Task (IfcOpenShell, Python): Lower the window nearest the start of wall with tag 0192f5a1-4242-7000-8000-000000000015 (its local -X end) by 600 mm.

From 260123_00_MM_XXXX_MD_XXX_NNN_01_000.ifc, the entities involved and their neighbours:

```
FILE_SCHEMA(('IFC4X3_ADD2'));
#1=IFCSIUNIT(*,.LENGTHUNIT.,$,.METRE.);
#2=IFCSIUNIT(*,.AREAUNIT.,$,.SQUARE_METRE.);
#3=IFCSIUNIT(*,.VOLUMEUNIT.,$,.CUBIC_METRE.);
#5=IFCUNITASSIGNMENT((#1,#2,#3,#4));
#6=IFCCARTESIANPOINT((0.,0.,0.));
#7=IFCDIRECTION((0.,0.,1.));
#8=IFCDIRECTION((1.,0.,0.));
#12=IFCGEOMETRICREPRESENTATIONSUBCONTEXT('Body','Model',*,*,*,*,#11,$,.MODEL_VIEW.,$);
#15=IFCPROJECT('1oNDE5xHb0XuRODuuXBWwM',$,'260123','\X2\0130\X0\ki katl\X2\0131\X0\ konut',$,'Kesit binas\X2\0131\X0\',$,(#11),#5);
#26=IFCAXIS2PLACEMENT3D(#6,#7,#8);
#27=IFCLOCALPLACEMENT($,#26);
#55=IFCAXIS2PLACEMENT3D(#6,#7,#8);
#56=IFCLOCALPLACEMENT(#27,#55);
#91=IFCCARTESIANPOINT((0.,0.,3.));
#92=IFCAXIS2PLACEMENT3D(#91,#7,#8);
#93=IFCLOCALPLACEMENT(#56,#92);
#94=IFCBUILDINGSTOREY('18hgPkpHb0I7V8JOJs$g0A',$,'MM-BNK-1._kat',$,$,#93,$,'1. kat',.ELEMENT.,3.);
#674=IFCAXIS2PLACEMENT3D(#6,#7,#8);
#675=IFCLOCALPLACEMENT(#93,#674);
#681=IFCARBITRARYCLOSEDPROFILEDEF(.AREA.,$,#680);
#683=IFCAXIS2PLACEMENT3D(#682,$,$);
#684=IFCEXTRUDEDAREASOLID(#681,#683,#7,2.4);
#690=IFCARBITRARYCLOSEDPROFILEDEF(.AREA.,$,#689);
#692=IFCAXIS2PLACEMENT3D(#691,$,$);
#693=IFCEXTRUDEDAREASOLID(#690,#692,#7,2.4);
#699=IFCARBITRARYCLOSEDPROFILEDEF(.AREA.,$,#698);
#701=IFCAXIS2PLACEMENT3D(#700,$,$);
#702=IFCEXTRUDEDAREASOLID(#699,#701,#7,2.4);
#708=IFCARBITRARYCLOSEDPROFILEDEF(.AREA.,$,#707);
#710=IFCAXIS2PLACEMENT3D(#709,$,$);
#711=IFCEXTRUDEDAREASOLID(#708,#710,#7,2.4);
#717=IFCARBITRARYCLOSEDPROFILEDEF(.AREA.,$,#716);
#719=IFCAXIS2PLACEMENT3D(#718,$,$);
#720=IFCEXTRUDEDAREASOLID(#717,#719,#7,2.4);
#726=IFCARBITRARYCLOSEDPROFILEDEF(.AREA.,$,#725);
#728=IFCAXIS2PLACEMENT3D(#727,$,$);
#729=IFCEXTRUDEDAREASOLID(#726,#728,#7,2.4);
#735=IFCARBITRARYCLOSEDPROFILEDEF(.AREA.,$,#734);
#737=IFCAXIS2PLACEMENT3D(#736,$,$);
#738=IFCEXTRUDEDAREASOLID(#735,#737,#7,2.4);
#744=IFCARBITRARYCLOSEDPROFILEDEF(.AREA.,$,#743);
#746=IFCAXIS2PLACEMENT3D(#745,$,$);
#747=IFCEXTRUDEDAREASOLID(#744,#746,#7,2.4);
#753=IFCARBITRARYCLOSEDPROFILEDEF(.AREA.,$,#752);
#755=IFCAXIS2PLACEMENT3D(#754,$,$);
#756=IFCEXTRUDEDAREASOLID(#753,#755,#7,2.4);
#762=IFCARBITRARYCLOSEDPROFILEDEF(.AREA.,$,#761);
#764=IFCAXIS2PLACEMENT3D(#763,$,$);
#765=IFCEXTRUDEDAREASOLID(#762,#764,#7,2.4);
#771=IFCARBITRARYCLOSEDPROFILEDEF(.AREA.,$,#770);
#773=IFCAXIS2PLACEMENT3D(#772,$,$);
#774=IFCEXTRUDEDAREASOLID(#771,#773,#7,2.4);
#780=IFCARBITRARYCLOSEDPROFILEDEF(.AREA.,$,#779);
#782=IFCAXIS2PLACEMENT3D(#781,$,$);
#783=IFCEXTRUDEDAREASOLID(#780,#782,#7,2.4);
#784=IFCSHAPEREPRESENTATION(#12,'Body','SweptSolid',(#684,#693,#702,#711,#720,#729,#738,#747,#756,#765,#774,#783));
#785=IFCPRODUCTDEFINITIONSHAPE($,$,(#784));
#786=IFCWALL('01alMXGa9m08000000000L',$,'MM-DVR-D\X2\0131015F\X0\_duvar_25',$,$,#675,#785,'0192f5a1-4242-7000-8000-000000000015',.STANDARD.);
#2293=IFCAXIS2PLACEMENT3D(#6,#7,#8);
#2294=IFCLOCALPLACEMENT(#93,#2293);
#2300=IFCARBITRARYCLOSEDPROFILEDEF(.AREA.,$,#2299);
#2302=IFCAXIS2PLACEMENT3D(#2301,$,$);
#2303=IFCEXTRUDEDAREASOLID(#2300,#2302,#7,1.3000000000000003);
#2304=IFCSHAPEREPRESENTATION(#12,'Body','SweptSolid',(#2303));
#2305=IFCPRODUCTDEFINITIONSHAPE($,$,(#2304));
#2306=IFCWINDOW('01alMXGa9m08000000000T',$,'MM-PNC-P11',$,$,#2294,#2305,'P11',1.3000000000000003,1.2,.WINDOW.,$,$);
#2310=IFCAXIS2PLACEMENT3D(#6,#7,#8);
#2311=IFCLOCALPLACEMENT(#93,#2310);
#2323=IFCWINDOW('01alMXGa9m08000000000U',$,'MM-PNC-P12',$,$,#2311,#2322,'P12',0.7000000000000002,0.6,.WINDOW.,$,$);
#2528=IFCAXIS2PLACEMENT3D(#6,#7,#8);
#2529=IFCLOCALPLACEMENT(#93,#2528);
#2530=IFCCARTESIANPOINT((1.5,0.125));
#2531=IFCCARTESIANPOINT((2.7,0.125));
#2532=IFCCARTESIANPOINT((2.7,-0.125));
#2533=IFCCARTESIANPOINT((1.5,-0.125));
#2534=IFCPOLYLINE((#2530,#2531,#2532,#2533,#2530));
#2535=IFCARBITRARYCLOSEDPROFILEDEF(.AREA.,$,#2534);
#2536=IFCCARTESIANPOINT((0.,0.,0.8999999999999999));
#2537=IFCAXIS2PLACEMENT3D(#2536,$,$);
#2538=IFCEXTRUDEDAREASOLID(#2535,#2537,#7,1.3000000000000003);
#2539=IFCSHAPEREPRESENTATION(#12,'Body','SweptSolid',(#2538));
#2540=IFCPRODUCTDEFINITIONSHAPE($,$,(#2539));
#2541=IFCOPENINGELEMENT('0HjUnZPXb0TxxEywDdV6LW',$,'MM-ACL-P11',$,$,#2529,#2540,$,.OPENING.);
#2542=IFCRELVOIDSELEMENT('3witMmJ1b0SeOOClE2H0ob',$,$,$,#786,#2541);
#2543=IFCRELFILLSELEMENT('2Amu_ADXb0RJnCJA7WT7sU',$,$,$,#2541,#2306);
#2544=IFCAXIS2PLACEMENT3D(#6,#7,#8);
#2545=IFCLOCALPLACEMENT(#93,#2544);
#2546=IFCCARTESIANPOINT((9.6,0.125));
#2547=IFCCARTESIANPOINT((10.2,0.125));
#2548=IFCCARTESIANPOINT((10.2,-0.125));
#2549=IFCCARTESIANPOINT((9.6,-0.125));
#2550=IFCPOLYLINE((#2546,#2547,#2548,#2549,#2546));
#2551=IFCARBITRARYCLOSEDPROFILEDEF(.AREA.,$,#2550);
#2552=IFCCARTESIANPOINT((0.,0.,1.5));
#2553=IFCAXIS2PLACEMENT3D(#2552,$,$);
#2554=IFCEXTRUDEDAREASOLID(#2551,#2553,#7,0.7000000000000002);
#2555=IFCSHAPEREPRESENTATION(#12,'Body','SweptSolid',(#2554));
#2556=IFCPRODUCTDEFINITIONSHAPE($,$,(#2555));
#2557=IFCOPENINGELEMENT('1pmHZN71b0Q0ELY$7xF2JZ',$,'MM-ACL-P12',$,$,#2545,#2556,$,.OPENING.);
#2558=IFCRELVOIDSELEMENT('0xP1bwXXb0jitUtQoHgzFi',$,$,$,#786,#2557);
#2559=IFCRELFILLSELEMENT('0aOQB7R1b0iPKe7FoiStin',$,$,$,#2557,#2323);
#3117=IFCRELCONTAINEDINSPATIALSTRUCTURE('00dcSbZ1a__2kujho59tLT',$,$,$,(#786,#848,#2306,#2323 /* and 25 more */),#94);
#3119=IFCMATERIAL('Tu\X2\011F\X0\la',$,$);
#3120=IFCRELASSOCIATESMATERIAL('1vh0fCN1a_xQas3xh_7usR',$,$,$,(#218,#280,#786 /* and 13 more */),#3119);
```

```python
import numpy as np
import ifcopenshell
import ifcopenshell.api.geometry
import ifcopenshell.util.placement
import ifcopenshell.util.unit

model = ifcopenshell.open("260123_00_MM_XXXX_MD_XXX_NNN_01_000.ifc")
unit_scale = ifcopenshell.util.unit.calculate_unit_scale(model)

window = model.by_id(2306)
opening = window.FillsVoids[0].RelatingOpeningElement
dz = -0.6 / unit_scale

shift = np.array([0.0, 0.0, dz])
# The window is not placed relative to its opening, so move both.
for product in (opening, window):
    matrix = ifcopenshell.util.placement.get_local_placement(product.ObjectPlacement)
    matrix[:3, 3] += shift
    ifcopenshell.api.geometry.edit_object_placement(model, product=product, matrix=matrix, is_si=False)

print(f"moved by {dz * unit_scale:+.3f} m")

model.write("260123_00_MM_XXXX_MD_XXX_NNN_01_000_updated.ifc")
```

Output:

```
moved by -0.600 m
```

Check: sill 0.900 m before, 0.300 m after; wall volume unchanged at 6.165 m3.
